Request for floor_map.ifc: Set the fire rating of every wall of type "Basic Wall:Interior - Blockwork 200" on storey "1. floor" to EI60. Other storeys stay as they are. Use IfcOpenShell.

First a look at what the model holds.

```python
import ifcopenshell
import ifcopenshell.util.element

model = ifcopenshell.open("floor_map.ifc")
print(model.schema)
storey = next(s for s in model.by_type("IfcBuildingStorey") if s.Name == "1. floor")
walls = [e for e in ifcopenshell.util.element.get_decomposition(storey) if e.is_a("IfcWall")]
seen = {}
for e in walls:
    element_type = ifcopenshell.util.element.get_type(e)
    key = (element_type.Name if element_type != e and element_type else None, ifcopenshell.util.element.get_pset(e, "Pset_WallCommon", "FireRating"))
    seen[key] = seen.get(key, 0) + 1
for (name, value), count in sorted(seen.items(), key=str):
    print(count, "x", name, "|", value)
```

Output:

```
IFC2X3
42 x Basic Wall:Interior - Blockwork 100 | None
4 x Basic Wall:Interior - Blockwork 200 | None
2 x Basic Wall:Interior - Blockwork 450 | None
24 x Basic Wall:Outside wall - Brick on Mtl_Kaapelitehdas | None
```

```python
import ifcopenshell
import ifcopenshell.api.pset
import ifcopenshell.util.element

model = ifcopenshell.open("floor_map.ifc")

storey = next(s for s in model.by_type("IfcBuildingStorey") if s.Name == "1. floor")
walls = [e for e in ifcopenshell.util.element.get_decomposition(storey) if e.is_a("IfcWall")]

count = 0
for e in walls:
    element_type = ifcopenshell.util.element.get_type(e)
    if element_type in (None, e) or element_type.Name != "Basic Wall:Interior - Blockwork 200":
        continue
    # add_pset returns the element's existing set when there is one.
    pset = ifcopenshell.api.pset.add_pset(model, product=e, name="Pset_WallCommon")
    ifcopenshell.api.pset.edit_pset(model, pset=pset, properties={"FireRating": "EI60"})
    count += 1

print(count, "walls updated")

model.write("floor_map_updated.ifc")
```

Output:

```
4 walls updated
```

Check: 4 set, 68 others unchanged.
